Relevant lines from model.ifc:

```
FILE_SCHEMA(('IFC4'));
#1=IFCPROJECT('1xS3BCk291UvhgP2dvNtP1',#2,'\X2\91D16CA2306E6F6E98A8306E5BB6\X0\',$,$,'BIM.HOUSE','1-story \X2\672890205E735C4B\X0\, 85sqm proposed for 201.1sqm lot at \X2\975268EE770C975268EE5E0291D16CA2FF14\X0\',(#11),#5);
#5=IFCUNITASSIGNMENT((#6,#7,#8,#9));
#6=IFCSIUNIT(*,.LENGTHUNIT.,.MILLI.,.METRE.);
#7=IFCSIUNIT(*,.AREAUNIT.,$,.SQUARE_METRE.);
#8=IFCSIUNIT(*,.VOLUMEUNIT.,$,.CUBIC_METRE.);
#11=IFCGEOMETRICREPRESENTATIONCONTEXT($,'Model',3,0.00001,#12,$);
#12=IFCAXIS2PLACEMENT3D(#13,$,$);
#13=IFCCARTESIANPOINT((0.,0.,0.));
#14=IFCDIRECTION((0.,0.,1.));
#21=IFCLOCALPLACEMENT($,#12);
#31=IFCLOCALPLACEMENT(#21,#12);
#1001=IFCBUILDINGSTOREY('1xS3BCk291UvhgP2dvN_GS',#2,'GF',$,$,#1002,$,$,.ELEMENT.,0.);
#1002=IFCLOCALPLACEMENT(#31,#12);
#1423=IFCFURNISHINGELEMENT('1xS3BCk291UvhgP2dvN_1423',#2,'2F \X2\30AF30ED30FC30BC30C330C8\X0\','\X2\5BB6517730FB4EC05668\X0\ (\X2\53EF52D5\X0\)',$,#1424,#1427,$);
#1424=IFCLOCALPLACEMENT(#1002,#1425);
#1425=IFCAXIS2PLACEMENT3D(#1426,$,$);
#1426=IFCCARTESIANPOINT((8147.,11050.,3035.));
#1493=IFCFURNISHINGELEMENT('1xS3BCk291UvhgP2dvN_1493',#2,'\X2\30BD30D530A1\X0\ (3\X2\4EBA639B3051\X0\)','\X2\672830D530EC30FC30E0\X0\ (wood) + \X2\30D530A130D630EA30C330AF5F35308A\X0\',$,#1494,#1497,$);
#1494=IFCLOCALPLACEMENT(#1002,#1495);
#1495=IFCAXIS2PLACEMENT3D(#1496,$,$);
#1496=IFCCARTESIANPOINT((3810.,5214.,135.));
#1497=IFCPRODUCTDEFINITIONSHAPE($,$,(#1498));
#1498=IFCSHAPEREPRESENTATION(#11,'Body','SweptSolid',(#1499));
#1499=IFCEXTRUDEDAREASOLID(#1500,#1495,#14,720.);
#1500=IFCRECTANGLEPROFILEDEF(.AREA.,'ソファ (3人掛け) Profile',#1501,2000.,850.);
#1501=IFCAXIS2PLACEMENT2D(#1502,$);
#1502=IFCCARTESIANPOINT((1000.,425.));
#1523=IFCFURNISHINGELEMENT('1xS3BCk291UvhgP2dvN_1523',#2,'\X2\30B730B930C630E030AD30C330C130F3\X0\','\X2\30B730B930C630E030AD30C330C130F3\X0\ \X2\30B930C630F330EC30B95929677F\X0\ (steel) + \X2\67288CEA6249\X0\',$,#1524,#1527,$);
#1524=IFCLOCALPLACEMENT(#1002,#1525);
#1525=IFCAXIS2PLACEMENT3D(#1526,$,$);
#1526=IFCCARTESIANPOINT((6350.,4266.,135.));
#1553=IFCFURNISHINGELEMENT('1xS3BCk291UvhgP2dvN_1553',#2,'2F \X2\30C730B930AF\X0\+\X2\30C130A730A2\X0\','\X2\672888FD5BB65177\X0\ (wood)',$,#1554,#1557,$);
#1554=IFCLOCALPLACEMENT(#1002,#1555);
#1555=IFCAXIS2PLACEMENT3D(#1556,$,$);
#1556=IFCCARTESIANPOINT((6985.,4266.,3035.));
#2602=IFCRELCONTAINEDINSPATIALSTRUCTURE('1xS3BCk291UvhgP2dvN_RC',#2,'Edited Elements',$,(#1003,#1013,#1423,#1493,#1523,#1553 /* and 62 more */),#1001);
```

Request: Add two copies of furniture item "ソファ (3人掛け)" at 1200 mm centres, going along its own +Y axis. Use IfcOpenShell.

```python
import ifcopenshell
import ifcopenshell.api.geometry
import ifcopenshell.api.root
import ifcopenshell.util.element
import ifcopenshell.util.placement
import ifcopenshell.util.unit

model = ifcopenshell.open("model.ifc")
unit_scale = ifcopenshell.util.unit.calculate_unit_scale(model)


def reuse_history(source, copy):
    """copy_class also copies each property set's owner history, people and application; keep the originals."""
    for rel in copy.IsDefinedBy:
        if rel.is_a("IfcRelDefinesByProperties") and (history := rel.RelatingPropertyDefinition.OwnerHistory):
            rel.RelatingPropertyDefinition.OwnerHistory = source.OwnerHistory
            ifcopenshell.util.element.remove_deep2(model, history)


source = model.by_guid("1xS3BCk291UvhgP2dvN_1493")
base = ifcopenshell.util.placement.get_local_placement(source.ObjectPlacement)
step = base[:3, 1] * 1.2 / unit_scale

for i in range(1, 3):
    copy = ifcopenshell.api.root.copy_class(model, product=source)
    copy.Representation = ifcopenshell.util.element.copy_deep(
        model, source.Representation, exclude=["IfcGeometricRepresentationContext", "IfcRepresentationMap"]
    )
    reuse_history(source, copy)
    matrix = base.copy()
    matrix[:3, 3] += i * step
    print("added at", matrix[:3, 3].round(3) + 0.0)
    ifcopenshell.api.geometry.edit_object_placement(model, product=copy, matrix=matrix, is_si=False)

model.write("model_v2.ifc")
```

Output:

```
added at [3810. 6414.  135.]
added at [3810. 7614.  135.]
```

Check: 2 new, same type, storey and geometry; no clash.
